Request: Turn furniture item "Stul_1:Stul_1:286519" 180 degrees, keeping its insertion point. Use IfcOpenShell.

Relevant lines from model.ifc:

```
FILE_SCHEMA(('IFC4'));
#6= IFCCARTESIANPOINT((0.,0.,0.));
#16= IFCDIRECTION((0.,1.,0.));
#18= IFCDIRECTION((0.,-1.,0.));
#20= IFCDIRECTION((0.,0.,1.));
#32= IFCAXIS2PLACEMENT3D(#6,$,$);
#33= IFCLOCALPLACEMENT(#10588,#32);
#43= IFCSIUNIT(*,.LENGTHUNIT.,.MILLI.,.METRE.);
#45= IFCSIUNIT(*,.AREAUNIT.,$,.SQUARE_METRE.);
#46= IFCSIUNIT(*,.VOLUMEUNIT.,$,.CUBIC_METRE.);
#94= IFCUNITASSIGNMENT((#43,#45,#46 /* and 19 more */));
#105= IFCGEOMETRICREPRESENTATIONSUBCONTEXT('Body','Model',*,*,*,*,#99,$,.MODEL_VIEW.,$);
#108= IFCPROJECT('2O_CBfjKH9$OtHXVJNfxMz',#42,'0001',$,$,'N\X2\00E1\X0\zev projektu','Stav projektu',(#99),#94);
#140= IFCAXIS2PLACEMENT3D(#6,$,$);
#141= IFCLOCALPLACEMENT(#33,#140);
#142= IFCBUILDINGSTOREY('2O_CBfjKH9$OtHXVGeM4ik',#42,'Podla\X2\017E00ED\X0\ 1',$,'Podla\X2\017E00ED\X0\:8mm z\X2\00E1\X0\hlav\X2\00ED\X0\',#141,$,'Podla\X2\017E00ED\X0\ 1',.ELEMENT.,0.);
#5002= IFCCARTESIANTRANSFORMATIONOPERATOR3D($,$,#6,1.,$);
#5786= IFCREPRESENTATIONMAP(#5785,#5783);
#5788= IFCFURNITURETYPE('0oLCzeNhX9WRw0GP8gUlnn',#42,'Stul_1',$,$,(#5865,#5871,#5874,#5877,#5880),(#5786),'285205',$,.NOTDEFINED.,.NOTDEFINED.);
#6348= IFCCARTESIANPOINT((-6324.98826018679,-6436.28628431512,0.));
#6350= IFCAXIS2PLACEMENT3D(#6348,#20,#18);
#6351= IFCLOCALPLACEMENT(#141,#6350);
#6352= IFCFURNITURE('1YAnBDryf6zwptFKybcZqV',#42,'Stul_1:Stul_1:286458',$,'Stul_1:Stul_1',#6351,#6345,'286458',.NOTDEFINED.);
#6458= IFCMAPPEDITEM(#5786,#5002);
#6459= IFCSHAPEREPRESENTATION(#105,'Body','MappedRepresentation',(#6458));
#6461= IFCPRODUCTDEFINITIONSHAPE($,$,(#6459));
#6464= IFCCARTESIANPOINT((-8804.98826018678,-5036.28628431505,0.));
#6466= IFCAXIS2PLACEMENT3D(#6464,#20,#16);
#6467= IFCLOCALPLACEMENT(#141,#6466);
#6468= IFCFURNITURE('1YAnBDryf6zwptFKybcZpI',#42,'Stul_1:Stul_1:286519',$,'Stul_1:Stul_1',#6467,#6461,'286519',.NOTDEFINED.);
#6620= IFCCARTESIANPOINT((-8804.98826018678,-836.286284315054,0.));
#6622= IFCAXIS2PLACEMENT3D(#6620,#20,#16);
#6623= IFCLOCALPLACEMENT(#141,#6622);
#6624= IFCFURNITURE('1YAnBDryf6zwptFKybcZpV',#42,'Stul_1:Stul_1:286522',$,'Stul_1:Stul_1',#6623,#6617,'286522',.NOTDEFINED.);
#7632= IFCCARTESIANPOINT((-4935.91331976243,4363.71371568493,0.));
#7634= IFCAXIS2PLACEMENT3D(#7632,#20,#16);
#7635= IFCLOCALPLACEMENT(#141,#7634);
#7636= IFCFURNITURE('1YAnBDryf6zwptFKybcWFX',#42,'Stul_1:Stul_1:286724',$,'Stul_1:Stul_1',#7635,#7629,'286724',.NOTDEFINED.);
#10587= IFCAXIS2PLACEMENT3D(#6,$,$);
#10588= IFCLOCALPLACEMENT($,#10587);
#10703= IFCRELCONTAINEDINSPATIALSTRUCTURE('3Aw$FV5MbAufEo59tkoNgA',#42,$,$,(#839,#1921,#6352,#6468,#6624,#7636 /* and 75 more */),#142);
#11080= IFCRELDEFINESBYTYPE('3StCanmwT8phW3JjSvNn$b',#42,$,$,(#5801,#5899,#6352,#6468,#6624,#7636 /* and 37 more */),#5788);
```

```python
import ifcopenshell
import ifcopenshell.api.geometry
import ifcopenshell.util.placement

model = ifcopenshell.open("model.ifc")

item = model.by_guid("1YAnBDryf6zwptFKybcZpI")
matrix = ifcopenshell.util.placement.get_local_placement(item.ObjectPlacement)
matrix = matrix @ ifcopenshell.util.placement.rotation(180, "Z")
ifcopenshell.api.geometry.edit_object_placement(model, product=item, matrix=matrix, is_si=False)

print(ifcopenshell.util.placement.get_local_placement(item.ObjectPlacement).round(3) + 0.0)

model.write("model_v2.ifc")
```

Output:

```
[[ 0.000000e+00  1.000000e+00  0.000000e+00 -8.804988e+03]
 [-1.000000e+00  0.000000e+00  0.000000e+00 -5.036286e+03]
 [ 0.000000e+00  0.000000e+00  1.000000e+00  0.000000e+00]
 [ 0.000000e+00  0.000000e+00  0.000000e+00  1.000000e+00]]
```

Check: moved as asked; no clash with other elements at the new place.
